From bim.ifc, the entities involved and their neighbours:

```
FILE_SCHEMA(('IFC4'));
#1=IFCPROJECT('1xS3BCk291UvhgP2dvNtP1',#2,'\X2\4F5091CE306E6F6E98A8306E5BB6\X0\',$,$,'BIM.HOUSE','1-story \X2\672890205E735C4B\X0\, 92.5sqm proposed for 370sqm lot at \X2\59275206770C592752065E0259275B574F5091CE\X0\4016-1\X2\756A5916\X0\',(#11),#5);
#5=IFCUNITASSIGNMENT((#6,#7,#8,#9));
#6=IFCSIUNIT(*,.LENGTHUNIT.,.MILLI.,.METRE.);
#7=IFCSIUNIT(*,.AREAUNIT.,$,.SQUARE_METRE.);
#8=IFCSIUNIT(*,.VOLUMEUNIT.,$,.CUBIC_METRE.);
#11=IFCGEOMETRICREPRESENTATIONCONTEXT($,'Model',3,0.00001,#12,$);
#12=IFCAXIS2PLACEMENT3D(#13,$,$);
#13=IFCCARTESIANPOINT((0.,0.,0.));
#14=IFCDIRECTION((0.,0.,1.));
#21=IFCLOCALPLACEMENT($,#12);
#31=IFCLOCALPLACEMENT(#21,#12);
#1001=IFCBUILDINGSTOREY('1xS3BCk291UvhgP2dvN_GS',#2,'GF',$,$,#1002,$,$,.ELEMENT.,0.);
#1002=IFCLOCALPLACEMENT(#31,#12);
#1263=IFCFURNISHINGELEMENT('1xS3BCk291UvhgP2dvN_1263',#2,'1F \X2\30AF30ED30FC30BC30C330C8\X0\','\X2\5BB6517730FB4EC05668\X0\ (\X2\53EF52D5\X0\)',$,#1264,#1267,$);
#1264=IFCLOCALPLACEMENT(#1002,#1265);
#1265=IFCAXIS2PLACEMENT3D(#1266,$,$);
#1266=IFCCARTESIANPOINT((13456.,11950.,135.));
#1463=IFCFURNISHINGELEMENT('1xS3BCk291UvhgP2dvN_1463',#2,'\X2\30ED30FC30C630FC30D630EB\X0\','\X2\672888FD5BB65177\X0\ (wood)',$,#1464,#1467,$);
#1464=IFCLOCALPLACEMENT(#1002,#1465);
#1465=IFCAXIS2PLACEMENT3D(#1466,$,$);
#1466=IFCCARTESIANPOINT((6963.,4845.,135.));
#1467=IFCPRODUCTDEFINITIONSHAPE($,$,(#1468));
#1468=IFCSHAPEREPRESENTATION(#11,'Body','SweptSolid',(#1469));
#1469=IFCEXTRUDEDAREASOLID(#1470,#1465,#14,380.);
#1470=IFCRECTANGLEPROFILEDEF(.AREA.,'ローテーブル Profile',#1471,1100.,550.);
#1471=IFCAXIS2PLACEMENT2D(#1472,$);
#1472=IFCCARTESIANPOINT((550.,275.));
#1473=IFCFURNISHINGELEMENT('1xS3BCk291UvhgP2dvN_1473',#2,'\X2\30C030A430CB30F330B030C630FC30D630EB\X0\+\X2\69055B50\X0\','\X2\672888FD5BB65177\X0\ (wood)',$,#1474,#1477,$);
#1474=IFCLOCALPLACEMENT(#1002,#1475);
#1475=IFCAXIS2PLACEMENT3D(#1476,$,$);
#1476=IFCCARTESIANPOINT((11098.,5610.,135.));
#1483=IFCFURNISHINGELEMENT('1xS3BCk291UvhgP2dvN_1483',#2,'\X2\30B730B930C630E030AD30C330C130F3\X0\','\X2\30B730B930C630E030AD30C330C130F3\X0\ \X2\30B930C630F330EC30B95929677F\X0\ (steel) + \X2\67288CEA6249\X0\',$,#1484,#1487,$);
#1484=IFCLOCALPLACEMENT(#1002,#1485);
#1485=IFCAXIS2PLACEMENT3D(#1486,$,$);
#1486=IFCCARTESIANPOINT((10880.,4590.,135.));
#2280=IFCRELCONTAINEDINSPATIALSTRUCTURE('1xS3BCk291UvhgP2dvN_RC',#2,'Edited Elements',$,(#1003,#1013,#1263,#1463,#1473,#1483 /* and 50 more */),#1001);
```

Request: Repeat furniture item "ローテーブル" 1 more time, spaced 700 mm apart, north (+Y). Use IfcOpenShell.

```python
import numpy as np
import ifcopenshell
import ifcopenshell.api.geometry
import ifcopenshell.api.root
import ifcopenshell.util.element
import ifcopenshell.util.placement

model = ifcopenshell.open("bim.ifc")


def reuse_history(source, copy):
    """copy_class also copies each property set's owner history, people and application; keep the originals."""
    for rel in copy.IsDefinedBy:
        if rel.is_a("IfcRelDefinesByProperties") and (history := rel.RelatingPropertyDefinition.OwnerHistory):
            rel.RelatingPropertyDefinition.OwnerHistory = source.OwnerHistory
            ifcopenshell.util.element.remove_deep2(model, history)


source = model.by_id(1463)
base = ifcopenshell.util.placement.get_local_placement(source.ObjectPlacement)
step = np.array([0.0, 1.0, 0.0]) * 700.0

for i in range(1, 2):
    copy = ifcopenshell.api.root.copy_class(model, product=source)
    copy.Representation = ifcopenshell.util.element.copy_deep(
        model, source.Representation, exclude=["IfcGeometricRepresentationContext", "IfcRepresentationMap"]
    )
    reuse_history(source, copy)
    matrix = base.copy()
    matrix[:3, 3] += i * step
    print("added at", matrix[:3, 3].round(3) + 0.0)
    ifcopenshell.api.geometry.edit_object_placement(model, product=copy, matrix=matrix, is_si=False)

model.write("bim_edited.ifc")
```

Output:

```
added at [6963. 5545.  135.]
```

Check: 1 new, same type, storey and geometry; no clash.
